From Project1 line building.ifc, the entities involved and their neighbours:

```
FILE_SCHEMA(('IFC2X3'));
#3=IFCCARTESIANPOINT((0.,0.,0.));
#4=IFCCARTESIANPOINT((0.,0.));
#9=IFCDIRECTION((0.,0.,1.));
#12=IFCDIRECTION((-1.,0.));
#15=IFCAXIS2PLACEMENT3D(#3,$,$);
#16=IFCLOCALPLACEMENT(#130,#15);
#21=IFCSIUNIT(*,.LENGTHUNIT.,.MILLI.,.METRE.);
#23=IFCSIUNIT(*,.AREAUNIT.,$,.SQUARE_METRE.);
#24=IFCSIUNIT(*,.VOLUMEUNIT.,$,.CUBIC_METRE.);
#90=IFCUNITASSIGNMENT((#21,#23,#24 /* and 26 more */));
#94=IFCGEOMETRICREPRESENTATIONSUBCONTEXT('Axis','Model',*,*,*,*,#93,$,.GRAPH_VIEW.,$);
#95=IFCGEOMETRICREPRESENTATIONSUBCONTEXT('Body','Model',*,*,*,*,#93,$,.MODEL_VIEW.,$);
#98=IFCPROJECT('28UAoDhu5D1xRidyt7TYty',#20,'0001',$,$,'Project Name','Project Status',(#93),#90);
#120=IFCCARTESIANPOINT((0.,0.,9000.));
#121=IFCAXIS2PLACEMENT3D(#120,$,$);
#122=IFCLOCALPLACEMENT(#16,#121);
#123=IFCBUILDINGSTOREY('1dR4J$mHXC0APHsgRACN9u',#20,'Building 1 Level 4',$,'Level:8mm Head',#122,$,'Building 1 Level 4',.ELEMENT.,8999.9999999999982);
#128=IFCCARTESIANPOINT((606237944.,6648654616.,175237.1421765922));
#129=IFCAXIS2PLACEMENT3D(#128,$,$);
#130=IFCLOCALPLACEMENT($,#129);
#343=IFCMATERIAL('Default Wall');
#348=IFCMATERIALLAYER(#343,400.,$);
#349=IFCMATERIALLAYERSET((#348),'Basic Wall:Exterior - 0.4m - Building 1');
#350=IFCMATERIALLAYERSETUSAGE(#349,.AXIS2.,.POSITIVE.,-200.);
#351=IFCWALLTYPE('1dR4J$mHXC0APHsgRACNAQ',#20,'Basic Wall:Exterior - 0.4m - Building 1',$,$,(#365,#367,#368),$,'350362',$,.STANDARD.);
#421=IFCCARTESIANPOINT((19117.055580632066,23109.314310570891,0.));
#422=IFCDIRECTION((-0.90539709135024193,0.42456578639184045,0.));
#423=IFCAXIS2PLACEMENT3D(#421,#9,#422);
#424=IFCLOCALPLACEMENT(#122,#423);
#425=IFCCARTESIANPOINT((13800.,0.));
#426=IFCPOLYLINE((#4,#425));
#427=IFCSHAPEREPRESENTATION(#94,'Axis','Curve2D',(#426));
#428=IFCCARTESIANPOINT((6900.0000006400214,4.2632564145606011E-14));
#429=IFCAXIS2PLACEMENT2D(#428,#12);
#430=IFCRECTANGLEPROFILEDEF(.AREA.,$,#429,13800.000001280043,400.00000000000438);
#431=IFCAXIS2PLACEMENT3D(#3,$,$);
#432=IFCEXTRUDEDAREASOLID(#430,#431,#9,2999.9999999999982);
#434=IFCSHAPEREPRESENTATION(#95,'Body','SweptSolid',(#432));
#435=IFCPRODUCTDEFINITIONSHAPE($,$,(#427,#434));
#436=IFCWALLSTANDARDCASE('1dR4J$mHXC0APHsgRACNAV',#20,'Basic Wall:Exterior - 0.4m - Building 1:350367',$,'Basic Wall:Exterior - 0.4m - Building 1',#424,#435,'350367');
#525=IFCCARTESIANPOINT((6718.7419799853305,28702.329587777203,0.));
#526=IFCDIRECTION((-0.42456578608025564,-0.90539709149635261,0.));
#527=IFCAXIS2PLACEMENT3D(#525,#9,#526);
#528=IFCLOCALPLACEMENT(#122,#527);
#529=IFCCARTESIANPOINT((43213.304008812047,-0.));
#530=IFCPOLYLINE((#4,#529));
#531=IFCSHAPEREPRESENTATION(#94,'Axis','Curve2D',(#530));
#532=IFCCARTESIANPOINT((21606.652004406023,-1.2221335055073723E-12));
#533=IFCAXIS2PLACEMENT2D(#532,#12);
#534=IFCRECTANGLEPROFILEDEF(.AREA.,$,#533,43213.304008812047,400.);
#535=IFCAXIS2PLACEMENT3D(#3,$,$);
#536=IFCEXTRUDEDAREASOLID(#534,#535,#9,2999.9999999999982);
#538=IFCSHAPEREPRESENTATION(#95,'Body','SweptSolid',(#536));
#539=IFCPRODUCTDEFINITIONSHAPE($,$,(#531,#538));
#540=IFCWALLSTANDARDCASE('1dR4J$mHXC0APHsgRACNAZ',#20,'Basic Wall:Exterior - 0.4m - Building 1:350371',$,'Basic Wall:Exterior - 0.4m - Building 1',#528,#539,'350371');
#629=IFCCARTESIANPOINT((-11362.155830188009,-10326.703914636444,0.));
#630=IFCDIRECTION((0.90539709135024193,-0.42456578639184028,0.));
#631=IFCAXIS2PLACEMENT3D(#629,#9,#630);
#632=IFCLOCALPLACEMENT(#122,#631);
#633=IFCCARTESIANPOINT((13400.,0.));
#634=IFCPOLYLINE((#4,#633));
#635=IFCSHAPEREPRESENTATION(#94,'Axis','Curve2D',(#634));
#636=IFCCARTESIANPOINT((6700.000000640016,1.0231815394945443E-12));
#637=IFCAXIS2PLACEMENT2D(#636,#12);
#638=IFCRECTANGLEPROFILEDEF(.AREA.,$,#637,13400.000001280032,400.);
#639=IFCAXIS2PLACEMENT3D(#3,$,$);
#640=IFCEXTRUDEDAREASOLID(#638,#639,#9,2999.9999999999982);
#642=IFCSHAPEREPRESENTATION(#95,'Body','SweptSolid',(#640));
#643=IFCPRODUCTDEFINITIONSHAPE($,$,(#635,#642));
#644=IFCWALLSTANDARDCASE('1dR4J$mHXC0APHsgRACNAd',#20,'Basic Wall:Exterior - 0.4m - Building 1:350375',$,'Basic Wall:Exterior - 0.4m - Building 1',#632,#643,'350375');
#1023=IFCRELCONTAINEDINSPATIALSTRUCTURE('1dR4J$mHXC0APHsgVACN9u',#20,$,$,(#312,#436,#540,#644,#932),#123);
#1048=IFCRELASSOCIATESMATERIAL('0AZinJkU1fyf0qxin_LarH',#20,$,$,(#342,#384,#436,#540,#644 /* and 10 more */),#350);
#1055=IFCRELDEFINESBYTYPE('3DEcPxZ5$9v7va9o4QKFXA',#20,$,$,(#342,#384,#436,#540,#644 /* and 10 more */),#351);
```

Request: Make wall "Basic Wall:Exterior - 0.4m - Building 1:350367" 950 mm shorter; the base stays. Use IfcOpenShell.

```python
import ifcopenshell
import ifcopenshell.geom
import ifcopenshell.util.representation
import ifcopenshell.util.shape
import ifcopenshell.util.unit

model = ifcopenshell.open("Project1 line building.ifc")
unit_scale = ifcopenshell.util.unit.calculate_unit_scale(model)
settings = ifcopenshell.geom.settings()


def volume(element):
    """Net volume in cubic metres, openings subtracted."""
    shape = ifcopenshell.geom.create_shape(settings, element)
    return ifcopenshell.util.shape.get_volume(shape.geometry)


wall = model.by_guid("1dR4J$mHXC0APHsgRACNAV")
before = volume(wall)

body = ifcopenshell.util.representation.get_representation(wall, "Model", "Body")
solid = body.Items[0]
old_height = solid.Depth
solid.Depth -= 0.95 / unit_scale
after = volume(wall)

print(f"height {old_height:g} -> {solid.Depth:g}, volume {before:.3f} -> {after:.3f} m3")

model.write("Project1 line building_v2.ifc")
```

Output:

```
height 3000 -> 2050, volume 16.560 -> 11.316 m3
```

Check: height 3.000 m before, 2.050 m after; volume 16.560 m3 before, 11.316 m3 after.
